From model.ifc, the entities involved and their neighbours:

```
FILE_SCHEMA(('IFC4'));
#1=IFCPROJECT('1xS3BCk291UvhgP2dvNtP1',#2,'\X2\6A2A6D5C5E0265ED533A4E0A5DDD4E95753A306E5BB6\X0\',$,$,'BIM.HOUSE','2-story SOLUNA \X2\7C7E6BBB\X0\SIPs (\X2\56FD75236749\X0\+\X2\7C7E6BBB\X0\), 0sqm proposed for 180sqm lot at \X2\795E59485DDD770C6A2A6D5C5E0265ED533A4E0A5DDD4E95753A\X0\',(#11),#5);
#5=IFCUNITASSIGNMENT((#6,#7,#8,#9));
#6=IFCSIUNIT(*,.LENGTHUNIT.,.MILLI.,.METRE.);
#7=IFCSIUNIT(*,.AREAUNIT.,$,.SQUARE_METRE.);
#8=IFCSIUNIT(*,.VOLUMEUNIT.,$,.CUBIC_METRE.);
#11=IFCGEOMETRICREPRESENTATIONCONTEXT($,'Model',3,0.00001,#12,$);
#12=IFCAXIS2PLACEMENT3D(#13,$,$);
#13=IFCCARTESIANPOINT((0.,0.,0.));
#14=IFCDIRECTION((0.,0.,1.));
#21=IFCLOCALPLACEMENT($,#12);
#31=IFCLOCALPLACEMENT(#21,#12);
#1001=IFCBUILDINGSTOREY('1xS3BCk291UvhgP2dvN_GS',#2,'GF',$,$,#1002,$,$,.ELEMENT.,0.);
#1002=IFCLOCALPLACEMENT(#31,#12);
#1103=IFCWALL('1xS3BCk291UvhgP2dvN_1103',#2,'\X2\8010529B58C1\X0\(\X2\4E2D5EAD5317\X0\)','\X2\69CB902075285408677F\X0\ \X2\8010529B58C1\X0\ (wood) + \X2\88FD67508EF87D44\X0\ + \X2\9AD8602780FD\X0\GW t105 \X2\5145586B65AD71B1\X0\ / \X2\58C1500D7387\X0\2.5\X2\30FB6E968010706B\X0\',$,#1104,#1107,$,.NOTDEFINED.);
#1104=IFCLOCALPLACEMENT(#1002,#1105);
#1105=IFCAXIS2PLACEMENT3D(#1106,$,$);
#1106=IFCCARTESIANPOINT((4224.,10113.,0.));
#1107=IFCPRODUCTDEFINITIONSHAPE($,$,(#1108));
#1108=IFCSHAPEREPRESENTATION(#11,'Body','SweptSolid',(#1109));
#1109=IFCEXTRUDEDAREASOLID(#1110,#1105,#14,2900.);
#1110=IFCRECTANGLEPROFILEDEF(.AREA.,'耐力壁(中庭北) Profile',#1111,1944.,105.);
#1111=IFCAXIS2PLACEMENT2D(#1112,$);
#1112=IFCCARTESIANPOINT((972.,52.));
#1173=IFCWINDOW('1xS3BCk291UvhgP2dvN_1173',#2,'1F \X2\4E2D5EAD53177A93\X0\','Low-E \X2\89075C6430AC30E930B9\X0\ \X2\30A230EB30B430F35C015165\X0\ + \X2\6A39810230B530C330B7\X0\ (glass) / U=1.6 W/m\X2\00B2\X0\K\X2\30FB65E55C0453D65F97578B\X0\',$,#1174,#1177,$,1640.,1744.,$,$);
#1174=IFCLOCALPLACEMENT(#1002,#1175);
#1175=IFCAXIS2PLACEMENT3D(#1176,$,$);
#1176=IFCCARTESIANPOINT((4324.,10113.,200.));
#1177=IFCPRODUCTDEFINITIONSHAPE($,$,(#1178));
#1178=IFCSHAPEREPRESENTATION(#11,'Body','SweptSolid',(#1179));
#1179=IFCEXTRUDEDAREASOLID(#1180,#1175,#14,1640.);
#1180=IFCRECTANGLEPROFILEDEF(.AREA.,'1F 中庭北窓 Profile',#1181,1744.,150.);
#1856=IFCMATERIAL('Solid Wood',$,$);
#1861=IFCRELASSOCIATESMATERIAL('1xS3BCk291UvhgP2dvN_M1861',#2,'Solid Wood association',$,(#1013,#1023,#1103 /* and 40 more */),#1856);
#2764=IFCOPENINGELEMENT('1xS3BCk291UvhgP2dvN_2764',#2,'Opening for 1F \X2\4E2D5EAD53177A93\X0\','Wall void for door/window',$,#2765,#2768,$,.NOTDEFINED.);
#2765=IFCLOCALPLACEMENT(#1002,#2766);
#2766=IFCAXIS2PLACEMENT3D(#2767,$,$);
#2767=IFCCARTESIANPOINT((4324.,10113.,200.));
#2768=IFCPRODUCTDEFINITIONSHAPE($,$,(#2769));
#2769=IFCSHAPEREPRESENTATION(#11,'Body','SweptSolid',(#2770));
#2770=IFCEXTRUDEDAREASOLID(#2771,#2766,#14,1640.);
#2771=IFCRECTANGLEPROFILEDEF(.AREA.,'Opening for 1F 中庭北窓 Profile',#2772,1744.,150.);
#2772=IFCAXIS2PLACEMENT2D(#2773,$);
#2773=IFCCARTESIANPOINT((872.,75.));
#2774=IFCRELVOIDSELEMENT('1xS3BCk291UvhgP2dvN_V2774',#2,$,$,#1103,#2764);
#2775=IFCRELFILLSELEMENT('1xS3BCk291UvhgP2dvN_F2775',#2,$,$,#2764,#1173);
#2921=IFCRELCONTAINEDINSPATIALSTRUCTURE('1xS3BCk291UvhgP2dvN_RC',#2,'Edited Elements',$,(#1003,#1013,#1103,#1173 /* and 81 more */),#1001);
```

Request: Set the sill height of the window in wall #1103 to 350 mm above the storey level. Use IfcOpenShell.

```python
import numpy as np
import ifcopenshell
import ifcopenshell.api.geometry
import ifcopenshell.geom
import ifcopenshell.util.element
import ifcopenshell.util.placement
import ifcopenshell.util.shape
import ifcopenshell.util.unit

model = ifcopenshell.open("model.ifc")
unit_scale = ifcopenshell.util.unit.calculate_unit_scale(model)

window = model.by_id(1173)
opening = window.FillsVoids[0].RelatingOpeningElement
storey = ifcopenshell.util.element.get_container(window, ifc_class="IfcBuildingStorey")
level = ifcopenshell.util.placement.get_local_placement(storey.ObjectPlacement)[2, 3]

# The opening's origin need not be at the sill, so measure its lowest point.
shape = ifcopenshell.geom.create_shape(ifcopenshell.geom.settings(), opening)
bottom = ifcopenshell.util.shape.get_shape_bottom_elevation(shape, shape.geometry) / unit_scale
dz = level + 350.0 - bottom

shift = np.array([0.0, 0.0, dz])
# The window is not placed relative to its opening, so move both.
for product in (opening, window):
    matrix = ifcopenshell.util.placement.get_local_placement(product.ObjectPlacement)
    matrix[:3, 3] += shift
    ifcopenshell.api.geometry.edit_object_placement(model, product=product, matrix=matrix, is_si=False)

print(f"moved by {dz * unit_scale:+.3f} m")

model.write("model_v2.ifc")
```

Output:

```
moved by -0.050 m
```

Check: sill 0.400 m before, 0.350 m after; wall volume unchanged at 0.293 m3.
